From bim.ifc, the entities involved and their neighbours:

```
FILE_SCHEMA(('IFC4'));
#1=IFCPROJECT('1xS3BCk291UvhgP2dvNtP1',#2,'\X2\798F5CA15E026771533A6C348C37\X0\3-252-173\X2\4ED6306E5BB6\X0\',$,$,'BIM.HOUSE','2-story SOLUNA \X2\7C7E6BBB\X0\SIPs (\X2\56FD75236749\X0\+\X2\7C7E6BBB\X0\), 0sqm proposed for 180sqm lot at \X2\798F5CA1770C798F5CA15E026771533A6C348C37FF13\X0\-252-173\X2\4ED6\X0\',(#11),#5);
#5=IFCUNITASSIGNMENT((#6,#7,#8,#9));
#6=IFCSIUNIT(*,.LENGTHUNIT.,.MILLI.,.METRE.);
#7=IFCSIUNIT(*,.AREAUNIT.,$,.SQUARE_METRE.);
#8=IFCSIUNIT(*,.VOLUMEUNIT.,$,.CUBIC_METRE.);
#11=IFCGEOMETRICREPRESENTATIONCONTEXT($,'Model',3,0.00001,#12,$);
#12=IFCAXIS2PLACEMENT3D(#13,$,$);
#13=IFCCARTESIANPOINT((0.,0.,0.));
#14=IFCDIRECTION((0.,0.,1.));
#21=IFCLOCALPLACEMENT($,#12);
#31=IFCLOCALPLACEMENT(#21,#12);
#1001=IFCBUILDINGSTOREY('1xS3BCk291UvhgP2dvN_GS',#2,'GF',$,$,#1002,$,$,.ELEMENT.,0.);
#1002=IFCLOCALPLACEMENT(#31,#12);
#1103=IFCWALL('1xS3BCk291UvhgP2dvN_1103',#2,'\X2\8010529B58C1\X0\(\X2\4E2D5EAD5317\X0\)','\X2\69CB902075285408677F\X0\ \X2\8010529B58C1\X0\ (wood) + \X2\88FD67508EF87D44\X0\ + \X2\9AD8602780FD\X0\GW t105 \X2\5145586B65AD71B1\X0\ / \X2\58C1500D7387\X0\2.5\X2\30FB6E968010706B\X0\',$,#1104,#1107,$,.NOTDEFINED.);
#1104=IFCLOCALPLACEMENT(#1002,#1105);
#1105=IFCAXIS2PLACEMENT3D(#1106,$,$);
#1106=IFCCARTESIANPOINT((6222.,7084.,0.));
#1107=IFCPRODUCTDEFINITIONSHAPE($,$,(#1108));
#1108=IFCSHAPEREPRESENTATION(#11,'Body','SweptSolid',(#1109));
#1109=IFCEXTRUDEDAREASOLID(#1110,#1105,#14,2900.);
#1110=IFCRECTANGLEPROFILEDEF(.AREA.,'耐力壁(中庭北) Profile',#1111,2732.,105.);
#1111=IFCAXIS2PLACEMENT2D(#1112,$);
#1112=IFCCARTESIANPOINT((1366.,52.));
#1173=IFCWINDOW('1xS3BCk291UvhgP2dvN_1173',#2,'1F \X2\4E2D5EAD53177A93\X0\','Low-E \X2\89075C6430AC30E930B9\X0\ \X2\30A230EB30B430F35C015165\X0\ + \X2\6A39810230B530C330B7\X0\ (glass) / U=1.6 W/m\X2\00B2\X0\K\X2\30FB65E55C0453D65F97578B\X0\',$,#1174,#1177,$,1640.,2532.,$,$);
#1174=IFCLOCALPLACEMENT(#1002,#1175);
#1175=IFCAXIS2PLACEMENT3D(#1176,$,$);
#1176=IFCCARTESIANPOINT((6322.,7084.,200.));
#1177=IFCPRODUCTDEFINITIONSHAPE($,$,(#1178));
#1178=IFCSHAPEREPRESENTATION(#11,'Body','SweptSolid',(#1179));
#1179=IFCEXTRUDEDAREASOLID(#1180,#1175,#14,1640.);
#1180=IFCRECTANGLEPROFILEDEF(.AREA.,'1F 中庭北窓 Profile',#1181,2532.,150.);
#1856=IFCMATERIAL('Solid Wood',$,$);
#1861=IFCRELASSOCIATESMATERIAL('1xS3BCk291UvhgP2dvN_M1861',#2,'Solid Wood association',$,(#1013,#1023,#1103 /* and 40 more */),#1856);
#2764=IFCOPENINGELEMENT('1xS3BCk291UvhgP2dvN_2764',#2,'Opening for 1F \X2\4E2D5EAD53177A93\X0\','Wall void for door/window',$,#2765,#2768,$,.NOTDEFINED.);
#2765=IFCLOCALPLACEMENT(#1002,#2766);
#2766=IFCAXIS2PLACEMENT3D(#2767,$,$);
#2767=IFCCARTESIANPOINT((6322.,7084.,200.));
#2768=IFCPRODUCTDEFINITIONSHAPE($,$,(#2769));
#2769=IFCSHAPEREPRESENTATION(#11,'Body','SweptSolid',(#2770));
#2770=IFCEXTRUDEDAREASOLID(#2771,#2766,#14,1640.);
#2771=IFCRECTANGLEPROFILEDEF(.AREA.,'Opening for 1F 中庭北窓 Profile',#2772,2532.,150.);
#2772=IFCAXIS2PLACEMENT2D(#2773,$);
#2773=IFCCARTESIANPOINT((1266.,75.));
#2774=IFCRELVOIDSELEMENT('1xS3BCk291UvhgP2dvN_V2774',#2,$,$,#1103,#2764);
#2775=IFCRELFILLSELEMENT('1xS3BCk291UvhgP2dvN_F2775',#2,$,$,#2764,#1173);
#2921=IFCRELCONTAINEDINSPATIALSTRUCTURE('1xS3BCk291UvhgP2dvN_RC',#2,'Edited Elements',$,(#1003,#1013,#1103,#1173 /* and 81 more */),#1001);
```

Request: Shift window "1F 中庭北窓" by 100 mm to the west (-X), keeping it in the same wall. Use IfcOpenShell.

```python
import ifcopenshell
import ifcopenshell.api.geometry
import ifcopenshell.util.placement

model = ifcopenshell.open("bim.ifc")

window = model.by_guid("1xS3BCk291UvhgP2dvN_1173")
opening = window.FillsVoids[0].RelatingOpeningElement
wall = opening.VoidsElements[0].RelatingBuildingElement

wall_matrix = ifcopenshell.util.placement.get_local_placement(wall.ObjectPlacement)
shift = wall_matrix[:3, 0] * -100.0
before = ifcopenshell.util.placement.get_local_placement(window.ObjectPlacement)[:3, 3].copy()

# The window is not placed relative to its opening, so move both.
for product in (opening, window):
    matrix = ifcopenshell.util.placement.get_local_placement(product.ObjectPlacement)
    matrix[:3, 3] += shift
    ifcopenshell.api.geometry.edit_object_placement(model, product=product, matrix=matrix, is_si=False)

after = ifcopenshell.util.placement.get_local_placement(window.ObjectPlacement)[:3, 3]
print("window moved by", (after - before).round(3) + 0.0)

model.write("bim_updated.ifc")
```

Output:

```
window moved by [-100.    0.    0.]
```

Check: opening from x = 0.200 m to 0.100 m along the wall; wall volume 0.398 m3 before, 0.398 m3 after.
